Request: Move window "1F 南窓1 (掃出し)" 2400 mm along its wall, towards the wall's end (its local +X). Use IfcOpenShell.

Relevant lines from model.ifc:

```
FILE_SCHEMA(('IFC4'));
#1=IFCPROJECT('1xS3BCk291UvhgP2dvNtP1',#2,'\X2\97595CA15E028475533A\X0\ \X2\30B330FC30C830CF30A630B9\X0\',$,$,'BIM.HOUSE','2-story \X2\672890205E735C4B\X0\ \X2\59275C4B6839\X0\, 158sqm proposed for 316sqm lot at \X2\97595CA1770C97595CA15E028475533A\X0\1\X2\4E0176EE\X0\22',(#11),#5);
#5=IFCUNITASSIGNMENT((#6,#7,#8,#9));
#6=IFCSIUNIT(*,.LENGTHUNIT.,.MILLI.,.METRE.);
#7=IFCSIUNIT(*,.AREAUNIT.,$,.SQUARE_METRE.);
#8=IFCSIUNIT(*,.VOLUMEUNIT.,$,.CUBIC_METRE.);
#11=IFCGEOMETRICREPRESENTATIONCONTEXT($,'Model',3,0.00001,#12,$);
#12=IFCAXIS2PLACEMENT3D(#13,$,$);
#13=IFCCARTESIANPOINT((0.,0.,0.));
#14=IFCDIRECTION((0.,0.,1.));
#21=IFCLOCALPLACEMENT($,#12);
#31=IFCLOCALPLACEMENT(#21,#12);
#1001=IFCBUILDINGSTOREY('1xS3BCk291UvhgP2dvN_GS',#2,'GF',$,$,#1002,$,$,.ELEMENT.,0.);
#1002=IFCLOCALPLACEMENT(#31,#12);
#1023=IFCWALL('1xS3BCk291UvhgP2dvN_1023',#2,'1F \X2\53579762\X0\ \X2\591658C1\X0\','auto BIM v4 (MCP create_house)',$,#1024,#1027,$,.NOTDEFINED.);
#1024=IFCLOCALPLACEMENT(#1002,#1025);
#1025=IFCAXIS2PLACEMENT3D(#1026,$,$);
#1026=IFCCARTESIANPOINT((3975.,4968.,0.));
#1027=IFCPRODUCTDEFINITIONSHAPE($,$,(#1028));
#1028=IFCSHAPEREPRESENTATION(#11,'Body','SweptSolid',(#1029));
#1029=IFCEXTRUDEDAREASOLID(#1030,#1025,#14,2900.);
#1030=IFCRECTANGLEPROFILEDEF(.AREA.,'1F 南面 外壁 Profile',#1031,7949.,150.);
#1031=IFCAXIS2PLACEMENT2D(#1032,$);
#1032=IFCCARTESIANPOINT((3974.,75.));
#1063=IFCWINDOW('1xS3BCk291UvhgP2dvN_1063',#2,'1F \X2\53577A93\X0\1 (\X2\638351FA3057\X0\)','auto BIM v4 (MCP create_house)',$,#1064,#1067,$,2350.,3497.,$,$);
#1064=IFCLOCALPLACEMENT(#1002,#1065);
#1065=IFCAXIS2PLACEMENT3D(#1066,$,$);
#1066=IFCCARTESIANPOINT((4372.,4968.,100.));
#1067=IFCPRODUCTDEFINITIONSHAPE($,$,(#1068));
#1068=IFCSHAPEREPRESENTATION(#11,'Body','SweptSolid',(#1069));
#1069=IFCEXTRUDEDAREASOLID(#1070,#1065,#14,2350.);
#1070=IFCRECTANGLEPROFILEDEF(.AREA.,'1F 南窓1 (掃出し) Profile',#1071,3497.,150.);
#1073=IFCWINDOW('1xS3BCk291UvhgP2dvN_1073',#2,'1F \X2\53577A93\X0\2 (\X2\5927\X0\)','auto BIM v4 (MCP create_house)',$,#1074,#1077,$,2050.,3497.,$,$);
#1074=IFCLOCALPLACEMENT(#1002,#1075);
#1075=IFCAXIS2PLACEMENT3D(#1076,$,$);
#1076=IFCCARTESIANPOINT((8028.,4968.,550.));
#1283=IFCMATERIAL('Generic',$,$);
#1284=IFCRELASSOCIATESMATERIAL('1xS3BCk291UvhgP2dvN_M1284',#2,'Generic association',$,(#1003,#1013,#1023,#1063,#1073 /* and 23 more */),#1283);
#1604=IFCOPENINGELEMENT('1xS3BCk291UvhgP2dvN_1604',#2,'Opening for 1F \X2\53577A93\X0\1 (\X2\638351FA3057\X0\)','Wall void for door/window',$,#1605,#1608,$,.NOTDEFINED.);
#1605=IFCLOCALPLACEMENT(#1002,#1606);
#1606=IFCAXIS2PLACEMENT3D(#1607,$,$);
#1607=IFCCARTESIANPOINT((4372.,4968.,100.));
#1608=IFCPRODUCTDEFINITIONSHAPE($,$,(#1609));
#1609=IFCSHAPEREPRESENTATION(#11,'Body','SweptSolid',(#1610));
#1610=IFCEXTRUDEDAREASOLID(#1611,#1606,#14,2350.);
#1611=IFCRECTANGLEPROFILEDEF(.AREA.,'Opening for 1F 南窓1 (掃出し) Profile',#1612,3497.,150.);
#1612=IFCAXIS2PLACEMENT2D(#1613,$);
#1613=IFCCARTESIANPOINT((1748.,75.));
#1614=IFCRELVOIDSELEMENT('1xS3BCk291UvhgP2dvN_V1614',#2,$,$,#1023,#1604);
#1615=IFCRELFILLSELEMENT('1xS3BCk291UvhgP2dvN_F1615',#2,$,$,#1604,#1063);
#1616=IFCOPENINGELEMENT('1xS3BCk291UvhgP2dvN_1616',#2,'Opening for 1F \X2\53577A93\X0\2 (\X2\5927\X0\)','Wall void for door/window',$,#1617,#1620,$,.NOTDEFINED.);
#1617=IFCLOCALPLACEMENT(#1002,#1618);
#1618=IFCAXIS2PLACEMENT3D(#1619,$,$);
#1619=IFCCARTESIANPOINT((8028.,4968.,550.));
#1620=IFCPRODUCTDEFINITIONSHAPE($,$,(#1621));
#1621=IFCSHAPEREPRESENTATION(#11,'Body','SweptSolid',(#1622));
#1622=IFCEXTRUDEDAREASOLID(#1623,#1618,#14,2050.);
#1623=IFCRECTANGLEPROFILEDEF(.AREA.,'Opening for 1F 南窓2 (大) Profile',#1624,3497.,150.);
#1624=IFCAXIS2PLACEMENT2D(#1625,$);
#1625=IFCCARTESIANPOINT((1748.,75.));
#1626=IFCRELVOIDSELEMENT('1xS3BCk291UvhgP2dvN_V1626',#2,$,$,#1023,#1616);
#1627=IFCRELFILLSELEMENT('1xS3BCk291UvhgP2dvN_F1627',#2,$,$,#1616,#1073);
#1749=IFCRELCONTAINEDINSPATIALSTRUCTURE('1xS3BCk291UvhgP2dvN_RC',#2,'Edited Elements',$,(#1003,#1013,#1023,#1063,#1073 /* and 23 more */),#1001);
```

```python
import ifcopenshell
import ifcopenshell.api.geometry
import ifcopenshell.util.placement
import ifcopenshell.util.unit

model = ifcopenshell.open("model.ifc")
unit_scale = ifcopenshell.util.unit.calculate_unit_scale(model)

window = model.by_id(1063)
opening = window.FillsVoids[0].RelatingOpeningElement
wall = opening.VoidsElements[0].RelatingBuildingElement

wall_matrix = ifcopenshell.util.placement.get_local_placement(wall.ObjectPlacement)
shift = wall_matrix[:3, 0] * 2.4 / unit_scale
before = ifcopenshell.util.placement.get_local_placement(window.ObjectPlacement)[:3, 3].copy()

# The window is not placed relative to its opening, so move both.
for product in (opening, window):
    matrix = ifcopenshell.util.placement.get_local_placement(product.ObjectPlacement)
    matrix[:3, 3] += shift
    ifcopenshell.api.geometry.edit_object_placement(model, product=product, matrix=matrix, is_si=False)

after = ifcopenshell.util.placement.get_local_placement(window.ObjectPlacement)[:3, 3]
print("window moved by", (after - before).round(3) + 0.0)

model.write("model-out.ifc")
```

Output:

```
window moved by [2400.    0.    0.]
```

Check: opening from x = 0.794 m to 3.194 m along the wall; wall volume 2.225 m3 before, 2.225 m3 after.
